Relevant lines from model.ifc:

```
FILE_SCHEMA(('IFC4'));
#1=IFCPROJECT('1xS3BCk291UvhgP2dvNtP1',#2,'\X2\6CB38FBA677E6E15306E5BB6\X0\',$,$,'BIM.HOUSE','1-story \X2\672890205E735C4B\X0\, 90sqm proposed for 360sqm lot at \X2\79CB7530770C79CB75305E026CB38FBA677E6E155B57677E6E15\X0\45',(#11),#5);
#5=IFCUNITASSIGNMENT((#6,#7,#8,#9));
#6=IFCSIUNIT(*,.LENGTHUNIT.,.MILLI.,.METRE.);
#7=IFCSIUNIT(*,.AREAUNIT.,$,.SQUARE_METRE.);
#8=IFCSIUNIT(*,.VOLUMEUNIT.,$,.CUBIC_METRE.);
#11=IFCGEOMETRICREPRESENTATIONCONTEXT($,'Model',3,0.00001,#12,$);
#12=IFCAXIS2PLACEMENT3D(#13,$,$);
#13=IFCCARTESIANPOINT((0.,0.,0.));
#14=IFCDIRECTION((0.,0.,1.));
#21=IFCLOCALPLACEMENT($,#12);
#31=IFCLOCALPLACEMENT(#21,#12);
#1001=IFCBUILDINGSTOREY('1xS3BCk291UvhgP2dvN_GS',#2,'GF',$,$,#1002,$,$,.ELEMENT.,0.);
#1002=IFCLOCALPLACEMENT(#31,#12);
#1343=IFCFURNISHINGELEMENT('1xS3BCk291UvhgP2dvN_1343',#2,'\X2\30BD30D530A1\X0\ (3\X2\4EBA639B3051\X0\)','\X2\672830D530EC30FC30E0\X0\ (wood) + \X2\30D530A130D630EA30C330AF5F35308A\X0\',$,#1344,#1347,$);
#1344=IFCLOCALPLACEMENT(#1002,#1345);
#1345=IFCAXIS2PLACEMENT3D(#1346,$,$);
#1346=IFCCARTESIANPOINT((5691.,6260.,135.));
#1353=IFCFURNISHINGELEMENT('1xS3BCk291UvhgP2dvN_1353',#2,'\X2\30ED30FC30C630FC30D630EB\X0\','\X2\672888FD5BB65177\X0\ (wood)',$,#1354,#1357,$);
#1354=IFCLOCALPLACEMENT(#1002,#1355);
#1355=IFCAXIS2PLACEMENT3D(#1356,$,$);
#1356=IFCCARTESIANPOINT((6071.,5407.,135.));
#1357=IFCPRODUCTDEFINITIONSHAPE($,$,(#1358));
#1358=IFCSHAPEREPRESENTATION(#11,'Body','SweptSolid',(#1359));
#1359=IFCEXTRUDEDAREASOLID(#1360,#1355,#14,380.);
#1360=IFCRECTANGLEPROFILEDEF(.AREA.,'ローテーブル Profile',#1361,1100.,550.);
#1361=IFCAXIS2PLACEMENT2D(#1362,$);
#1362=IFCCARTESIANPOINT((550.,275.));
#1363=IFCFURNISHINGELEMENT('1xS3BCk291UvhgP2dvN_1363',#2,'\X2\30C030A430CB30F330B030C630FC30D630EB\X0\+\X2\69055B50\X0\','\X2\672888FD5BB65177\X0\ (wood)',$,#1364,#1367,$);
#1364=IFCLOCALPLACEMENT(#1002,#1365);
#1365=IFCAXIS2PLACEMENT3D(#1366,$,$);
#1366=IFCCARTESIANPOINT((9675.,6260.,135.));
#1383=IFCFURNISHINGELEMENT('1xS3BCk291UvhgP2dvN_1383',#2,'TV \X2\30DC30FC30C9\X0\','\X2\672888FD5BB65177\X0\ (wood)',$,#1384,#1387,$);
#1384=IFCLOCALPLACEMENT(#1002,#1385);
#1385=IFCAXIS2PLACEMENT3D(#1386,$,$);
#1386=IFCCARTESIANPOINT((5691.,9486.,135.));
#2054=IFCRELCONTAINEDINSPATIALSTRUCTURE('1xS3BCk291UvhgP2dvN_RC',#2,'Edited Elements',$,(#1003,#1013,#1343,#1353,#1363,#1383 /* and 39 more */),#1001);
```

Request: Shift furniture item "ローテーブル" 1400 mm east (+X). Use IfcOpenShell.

```python
import ifcopenshell
import ifcopenshell.api.geometry
import ifcopenshell.util.placement
import ifcopenshell.util.unit

model = ifcopenshell.open("model.ifc")
unit_scale = ifcopenshell.util.unit.calculate_unit_scale(model)

item = model.by_id(1353)
matrix = ifcopenshell.util.placement.get_local_placement(item.ObjectPlacement)
matrix[0, 3] += 1.4 / unit_scale
ifcopenshell.api.geometry.edit_object_placement(model, product=item, matrix=matrix, is_si=False)

print(ifcopenshell.util.placement.get_local_placement(item.ObjectPlacement).round(3) + 0.0)

model.write("model_updated.ifc")
```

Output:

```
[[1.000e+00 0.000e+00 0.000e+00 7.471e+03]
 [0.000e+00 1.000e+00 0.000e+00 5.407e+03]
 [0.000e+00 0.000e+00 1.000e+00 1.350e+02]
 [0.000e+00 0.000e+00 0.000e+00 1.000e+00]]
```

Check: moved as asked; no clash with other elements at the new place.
